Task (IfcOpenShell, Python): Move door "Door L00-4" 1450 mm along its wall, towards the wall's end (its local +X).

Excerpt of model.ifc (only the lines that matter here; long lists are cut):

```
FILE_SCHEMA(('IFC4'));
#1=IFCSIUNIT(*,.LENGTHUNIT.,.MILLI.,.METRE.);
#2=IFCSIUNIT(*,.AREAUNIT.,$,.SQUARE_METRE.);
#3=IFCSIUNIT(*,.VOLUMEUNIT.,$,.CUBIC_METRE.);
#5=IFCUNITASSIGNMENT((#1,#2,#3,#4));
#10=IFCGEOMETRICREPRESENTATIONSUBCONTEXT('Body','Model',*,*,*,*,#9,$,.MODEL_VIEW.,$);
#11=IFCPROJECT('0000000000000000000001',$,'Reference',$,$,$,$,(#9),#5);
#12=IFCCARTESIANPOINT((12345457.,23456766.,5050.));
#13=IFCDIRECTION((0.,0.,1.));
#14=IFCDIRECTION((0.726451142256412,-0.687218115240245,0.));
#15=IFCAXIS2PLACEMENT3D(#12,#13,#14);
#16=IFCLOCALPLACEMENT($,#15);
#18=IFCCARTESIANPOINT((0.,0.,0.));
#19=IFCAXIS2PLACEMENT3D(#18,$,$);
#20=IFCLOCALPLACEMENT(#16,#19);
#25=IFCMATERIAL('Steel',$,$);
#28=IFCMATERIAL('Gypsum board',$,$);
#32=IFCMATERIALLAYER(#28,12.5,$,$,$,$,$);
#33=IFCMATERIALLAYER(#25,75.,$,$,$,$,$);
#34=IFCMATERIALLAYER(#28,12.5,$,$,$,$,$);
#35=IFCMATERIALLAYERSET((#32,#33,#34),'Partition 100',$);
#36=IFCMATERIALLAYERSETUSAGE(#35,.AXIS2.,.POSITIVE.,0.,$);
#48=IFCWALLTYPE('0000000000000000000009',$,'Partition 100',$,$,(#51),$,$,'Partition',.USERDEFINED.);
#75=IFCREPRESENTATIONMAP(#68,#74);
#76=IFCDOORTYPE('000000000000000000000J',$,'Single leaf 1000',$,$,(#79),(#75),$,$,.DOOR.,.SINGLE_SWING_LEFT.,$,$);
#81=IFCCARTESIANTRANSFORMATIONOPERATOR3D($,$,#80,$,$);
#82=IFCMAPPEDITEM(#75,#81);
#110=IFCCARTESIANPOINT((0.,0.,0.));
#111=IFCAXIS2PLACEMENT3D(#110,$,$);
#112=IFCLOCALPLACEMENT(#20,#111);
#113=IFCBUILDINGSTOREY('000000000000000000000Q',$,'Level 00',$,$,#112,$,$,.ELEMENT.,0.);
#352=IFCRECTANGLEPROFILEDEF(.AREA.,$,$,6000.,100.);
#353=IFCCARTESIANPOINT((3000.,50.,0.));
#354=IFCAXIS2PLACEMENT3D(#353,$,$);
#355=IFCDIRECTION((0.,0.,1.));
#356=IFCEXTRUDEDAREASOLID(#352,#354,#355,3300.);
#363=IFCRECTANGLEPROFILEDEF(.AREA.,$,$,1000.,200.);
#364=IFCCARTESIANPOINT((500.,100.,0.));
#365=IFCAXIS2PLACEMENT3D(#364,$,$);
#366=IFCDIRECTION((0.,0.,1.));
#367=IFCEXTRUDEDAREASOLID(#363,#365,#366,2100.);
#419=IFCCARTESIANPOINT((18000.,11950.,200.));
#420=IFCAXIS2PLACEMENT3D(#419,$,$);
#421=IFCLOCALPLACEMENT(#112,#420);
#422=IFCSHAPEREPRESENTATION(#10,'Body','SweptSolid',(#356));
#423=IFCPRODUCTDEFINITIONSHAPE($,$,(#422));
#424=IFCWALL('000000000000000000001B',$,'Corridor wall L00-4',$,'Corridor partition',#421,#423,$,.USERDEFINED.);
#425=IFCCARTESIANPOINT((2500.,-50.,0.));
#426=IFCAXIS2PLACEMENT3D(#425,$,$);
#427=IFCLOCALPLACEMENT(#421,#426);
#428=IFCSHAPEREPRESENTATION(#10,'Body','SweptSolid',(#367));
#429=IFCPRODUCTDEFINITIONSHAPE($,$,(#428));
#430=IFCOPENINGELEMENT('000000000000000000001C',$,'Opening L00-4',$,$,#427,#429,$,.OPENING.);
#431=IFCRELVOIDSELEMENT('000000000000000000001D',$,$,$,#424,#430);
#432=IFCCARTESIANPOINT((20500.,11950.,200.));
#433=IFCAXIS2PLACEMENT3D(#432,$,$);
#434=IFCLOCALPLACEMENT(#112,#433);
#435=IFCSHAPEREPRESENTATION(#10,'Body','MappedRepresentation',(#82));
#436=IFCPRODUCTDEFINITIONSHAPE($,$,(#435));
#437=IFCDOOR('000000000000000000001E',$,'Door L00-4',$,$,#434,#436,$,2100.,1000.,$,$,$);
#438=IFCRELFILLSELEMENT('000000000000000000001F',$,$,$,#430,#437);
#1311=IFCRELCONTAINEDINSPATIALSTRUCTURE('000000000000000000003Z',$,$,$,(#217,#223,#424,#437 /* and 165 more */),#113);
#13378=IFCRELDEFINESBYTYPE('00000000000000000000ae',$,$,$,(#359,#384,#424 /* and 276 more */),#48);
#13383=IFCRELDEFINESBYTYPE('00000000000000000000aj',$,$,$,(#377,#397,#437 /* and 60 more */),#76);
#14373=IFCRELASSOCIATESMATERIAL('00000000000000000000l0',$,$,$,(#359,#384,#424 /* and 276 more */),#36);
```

```python
import ifcopenshell
import ifcopenshell.api.geometry
import ifcopenshell.util.placement
import ifcopenshell.util.unit

model = ifcopenshell.open("model.ifc")
unit_scale = ifcopenshell.util.unit.calculate_unit_scale(model)

door = model.by_guid("000000000000000000001E")
opening = door.FillsVoids[0].RelatingOpeningElement
wall = opening.VoidsElements[0].RelatingBuildingElement

wall_matrix = ifcopenshell.util.placement.get_local_placement(wall.ObjectPlacement)
shift = wall_matrix[:3, 0] * 1.45 / unit_scale
before = ifcopenshell.util.placement.get_local_placement(door.ObjectPlacement)[:3, 3].copy()

# The door is not placed relative to its opening, so move both.
for product in (opening, door):
    matrix = ifcopenshell.util.placement.get_local_placement(product.ObjectPlacement)
    matrix[:3, 3] += shift
    ifcopenshell.api.geometry.edit_object_placement(model, product=product, matrix=matrix, is_si=False)

after = ifcopenshell.util.placement.get_local_placement(door.ObjectPlacement)[:3, 3]
print("door moved by", (after - before).round(3) + 0.0)

model.write("model_v2.ifc")
```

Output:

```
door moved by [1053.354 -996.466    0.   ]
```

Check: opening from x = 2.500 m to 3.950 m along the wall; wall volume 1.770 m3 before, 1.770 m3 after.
